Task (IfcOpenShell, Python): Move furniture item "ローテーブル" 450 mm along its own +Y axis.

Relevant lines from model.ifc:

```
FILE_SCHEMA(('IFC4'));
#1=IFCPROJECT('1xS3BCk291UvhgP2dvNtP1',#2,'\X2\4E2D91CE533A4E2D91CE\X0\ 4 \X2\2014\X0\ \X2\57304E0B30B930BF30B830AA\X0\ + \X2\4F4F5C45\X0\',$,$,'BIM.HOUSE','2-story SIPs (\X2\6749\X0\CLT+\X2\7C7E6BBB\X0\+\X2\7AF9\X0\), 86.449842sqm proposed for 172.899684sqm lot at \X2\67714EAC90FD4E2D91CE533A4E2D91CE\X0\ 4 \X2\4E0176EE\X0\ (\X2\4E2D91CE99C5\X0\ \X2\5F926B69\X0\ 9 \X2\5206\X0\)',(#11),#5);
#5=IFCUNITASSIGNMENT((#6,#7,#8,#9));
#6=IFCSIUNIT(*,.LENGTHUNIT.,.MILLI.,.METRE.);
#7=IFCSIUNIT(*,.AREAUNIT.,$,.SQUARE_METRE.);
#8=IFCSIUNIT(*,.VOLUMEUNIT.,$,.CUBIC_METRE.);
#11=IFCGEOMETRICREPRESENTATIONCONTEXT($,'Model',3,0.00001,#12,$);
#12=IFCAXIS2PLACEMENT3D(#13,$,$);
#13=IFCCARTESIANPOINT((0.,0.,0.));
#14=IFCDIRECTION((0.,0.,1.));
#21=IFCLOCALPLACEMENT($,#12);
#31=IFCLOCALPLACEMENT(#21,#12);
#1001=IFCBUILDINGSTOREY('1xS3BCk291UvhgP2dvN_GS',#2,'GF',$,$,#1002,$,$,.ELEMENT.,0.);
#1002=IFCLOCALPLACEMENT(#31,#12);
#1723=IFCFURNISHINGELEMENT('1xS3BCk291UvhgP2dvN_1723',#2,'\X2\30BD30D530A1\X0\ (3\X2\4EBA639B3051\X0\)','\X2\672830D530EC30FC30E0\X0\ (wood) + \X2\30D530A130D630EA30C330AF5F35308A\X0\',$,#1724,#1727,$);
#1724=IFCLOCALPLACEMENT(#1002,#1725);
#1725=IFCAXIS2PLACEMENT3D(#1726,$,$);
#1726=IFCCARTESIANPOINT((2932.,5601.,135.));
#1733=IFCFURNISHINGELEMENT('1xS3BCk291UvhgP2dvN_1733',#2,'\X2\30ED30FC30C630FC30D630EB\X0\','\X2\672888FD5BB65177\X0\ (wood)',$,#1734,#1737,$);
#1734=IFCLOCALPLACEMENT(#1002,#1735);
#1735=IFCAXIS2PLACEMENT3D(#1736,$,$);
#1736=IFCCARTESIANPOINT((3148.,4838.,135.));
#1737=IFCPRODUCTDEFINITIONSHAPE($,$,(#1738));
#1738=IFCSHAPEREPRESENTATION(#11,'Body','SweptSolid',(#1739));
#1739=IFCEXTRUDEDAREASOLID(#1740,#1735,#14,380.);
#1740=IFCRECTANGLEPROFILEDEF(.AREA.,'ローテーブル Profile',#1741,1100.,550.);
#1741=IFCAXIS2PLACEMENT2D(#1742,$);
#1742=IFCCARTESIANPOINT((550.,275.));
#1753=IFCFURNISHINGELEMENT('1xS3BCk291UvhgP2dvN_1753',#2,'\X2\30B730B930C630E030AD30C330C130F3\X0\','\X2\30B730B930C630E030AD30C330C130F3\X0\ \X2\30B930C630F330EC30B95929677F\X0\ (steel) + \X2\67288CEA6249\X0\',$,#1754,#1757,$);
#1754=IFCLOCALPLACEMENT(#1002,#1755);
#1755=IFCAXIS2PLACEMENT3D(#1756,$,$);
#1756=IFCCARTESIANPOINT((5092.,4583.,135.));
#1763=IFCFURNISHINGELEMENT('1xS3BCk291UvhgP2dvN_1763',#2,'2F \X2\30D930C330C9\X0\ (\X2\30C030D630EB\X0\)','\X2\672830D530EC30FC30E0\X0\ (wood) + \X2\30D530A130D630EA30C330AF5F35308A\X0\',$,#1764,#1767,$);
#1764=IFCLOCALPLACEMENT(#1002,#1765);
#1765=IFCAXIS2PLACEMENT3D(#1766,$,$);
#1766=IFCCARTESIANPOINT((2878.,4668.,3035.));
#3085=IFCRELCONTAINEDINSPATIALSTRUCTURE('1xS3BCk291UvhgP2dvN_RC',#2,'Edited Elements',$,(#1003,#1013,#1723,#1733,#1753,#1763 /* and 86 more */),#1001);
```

```python
import ifcopenshell
import ifcopenshell.api.geometry
import ifcopenshell.util.placement
import ifcopenshell.util.unit

model = ifcopenshell.open("model.ifc")
unit_scale = ifcopenshell.util.unit.calculate_unit_scale(model)

item = model.by_guid("1xS3BCk291UvhgP2dvN_1733")
matrix = ifcopenshell.util.placement.get_local_placement(item.ObjectPlacement)
matrix[:3, 3] += matrix[:3, 1] * 0.45 / unit_scale
ifcopenshell.api.geometry.edit_object_placement(model, product=item, matrix=matrix, is_si=False)

print(ifcopenshell.util.placement.get_local_placement(item.ObjectPlacement).round(3) + 0.0)

model.write("model_updated.ifc")
```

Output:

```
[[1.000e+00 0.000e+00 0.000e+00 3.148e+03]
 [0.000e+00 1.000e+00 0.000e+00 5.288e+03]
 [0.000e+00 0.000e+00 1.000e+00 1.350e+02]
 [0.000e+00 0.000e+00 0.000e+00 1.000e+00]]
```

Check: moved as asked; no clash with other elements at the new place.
